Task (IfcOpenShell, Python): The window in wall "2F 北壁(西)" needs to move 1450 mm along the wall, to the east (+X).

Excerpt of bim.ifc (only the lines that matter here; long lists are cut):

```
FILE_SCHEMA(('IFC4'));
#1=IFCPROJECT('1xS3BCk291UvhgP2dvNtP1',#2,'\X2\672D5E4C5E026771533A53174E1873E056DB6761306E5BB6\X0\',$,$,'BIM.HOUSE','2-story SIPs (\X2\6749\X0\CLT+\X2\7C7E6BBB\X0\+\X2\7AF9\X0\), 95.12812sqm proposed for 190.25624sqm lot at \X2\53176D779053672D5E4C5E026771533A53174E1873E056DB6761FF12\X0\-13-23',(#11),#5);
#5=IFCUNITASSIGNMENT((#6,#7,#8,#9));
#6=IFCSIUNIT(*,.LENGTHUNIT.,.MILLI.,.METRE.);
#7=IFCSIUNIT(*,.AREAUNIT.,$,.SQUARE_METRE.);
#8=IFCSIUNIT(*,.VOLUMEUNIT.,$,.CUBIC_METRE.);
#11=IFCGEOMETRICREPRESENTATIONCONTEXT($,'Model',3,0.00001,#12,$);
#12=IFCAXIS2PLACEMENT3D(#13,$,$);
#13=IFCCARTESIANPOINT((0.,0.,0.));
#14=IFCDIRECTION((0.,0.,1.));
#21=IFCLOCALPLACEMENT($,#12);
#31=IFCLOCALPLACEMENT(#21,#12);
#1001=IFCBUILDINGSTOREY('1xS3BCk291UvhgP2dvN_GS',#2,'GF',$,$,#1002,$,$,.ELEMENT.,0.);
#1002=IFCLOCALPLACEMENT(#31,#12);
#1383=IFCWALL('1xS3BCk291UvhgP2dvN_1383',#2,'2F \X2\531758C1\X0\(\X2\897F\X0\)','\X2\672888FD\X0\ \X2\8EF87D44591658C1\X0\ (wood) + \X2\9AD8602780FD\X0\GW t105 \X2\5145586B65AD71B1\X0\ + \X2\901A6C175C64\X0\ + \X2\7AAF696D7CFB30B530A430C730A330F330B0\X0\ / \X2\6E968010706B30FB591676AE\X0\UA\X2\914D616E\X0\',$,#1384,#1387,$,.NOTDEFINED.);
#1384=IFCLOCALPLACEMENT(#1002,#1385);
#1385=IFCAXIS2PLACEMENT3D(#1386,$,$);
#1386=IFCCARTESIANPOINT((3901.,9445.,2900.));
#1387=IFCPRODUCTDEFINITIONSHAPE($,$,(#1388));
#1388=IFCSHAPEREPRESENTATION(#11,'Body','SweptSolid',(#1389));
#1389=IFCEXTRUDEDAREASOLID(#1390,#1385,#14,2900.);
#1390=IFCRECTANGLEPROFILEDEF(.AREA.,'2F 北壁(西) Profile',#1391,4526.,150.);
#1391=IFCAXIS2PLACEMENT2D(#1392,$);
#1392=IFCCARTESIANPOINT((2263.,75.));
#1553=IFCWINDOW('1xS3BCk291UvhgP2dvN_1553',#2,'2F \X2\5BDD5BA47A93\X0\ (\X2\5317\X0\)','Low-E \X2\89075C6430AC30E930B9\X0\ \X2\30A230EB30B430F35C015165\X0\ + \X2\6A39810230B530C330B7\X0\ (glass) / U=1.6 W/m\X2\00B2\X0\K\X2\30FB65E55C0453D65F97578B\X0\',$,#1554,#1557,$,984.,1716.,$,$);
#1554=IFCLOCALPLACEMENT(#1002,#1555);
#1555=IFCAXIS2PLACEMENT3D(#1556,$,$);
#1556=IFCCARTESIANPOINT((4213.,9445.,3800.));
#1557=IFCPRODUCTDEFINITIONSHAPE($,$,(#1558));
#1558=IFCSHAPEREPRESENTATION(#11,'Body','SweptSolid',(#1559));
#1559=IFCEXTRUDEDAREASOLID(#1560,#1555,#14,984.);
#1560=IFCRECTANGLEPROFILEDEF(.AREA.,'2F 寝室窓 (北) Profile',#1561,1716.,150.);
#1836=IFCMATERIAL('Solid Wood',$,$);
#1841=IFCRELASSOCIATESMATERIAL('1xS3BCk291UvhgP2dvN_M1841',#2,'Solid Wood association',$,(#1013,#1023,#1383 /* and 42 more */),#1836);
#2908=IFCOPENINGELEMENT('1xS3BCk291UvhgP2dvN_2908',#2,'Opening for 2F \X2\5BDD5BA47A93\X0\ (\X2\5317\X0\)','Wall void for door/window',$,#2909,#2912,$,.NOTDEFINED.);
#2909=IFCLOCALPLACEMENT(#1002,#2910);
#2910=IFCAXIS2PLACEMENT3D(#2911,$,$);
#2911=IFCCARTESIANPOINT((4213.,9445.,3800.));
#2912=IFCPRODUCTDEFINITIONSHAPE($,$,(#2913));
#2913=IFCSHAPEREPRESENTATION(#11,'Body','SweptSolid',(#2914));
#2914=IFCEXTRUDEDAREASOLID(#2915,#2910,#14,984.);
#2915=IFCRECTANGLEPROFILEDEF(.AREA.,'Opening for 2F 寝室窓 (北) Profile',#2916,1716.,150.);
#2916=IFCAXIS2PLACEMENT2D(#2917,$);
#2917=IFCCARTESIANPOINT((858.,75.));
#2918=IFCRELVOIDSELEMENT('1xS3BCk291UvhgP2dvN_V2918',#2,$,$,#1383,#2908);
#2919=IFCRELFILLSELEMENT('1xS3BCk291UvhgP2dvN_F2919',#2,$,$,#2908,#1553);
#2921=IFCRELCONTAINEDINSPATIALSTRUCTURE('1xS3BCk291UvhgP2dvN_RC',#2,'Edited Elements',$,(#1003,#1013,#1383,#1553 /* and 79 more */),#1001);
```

```python
import ifcopenshell
import ifcopenshell.api.geometry
import ifcopenshell.util.placement

model = ifcopenshell.open("bim.ifc")

window = model.by_id(1553)
opening = window.FillsVoids[0].RelatingOpeningElement
wall = opening.VoidsElements[0].RelatingBuildingElement

wall_matrix = ifcopenshell.util.placement.get_local_placement(wall.ObjectPlacement)
shift = wall_matrix[:3, 0] * 1450.0
before = ifcopenshell.util.placement.get_local_placement(window.ObjectPlacement)[:3, 3].copy()

# The window is not placed relative to its opening, so move both.
for product in (opening, window):
    matrix = ifcopenshell.util.placement.get_local_placement(product.ObjectPlacement)
    matrix[:3, 3] += shift
    ifcopenshell.api.geometry.edit_object_placement(model, product=product, matrix=matrix, is_si=False)

after = ifcopenshell.util.placement.get_local_placement(window.ObjectPlacement)[:3, 3]
print("window moved by", (after - before).round(3) + 0.0)

model.write("bim_updated.ifc")
```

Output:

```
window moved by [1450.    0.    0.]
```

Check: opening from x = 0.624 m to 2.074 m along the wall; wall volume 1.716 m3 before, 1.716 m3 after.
